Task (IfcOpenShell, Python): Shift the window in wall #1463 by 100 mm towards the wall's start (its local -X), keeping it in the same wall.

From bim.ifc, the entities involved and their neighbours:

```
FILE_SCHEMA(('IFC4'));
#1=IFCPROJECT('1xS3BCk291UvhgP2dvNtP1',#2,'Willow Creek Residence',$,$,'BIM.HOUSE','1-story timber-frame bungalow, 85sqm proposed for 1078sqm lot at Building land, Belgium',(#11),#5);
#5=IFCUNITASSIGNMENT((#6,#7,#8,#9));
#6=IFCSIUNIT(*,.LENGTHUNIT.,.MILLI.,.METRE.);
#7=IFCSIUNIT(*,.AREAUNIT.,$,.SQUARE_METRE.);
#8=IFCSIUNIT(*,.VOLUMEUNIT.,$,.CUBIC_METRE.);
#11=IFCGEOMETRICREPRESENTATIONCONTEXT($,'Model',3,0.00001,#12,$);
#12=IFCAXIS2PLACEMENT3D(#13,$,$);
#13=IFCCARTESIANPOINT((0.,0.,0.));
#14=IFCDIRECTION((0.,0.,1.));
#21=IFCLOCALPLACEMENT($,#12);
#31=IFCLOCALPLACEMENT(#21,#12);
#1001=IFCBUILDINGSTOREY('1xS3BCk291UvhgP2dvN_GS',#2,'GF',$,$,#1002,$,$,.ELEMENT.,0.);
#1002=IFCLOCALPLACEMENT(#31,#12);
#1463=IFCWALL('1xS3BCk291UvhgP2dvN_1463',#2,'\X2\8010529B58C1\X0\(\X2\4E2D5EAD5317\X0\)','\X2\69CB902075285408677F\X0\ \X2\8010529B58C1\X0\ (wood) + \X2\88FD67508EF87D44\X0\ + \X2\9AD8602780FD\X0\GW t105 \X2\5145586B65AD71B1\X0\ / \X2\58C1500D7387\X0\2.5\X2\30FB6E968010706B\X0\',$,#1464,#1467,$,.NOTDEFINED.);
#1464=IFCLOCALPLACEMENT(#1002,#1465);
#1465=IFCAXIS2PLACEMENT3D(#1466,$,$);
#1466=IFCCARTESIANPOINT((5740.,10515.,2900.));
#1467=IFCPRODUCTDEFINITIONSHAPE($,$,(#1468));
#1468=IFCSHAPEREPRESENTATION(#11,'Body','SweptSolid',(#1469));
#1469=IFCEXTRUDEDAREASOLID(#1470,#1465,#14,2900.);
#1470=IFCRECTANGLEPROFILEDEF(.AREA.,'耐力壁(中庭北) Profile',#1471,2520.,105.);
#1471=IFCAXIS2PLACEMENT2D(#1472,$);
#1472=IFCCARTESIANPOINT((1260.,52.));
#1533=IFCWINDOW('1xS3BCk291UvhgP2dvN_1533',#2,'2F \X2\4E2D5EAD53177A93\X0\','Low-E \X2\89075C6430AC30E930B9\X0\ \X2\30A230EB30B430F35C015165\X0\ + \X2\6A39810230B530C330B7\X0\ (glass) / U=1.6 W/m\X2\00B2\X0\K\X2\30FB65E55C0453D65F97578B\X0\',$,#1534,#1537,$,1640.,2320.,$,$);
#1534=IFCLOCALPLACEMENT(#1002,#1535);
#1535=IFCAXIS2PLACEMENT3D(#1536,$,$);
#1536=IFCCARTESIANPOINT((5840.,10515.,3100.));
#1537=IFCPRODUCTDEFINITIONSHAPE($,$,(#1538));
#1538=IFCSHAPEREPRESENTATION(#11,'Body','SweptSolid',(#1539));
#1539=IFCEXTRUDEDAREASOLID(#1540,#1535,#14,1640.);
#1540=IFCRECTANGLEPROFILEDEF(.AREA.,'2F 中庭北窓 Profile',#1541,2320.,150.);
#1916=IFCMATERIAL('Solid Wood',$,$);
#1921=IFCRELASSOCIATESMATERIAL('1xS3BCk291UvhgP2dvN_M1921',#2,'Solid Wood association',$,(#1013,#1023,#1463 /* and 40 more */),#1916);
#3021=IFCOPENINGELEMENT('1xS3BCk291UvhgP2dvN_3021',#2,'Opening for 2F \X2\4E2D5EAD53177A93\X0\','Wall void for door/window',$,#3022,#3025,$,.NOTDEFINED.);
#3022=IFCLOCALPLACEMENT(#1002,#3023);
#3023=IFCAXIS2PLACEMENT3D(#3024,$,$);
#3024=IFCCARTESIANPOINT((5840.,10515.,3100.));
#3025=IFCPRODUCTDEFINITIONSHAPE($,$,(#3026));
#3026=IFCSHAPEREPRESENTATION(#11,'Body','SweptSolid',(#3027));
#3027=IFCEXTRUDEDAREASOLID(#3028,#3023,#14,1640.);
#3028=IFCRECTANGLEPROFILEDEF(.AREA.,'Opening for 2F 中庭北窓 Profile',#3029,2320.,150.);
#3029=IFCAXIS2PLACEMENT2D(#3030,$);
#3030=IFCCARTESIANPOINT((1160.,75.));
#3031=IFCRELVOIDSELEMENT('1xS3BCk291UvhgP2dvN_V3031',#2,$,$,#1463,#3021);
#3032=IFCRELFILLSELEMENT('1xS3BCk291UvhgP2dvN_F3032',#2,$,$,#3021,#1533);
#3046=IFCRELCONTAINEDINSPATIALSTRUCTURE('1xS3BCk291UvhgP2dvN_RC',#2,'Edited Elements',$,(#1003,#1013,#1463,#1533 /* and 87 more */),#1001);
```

```python
import ifcopenshell
import ifcopenshell.api.geometry
import ifcopenshell.util.placement
import ifcopenshell.util.unit

model = ifcopenshell.open("bim.ifc")
unit_scale = ifcopenshell.util.unit.calculate_unit_scale(model)

window = model.by_guid("1xS3BCk291UvhgP2dvN_1533")
opening = window.FillsVoids[0].RelatingOpeningElement
wall = opening.VoidsElements[0].RelatingBuildingElement

wall_matrix = ifcopenshell.util.placement.get_local_placement(wall.ObjectPlacement)
shift = wall_matrix[:3, 0] * -0.1 / unit_scale
before = ifcopenshell.util.placement.get_local_placement(window.ObjectPlacement)[:3, 3].copy()

# The window is not placed relative to its opening, so move both.
for product in (opening, window):
    matrix = ifcopenshell.util.placement.get_local_placement(product.ObjectPlacement)
    matrix[:3, 3] += shift
    ifcopenshell.api.geometry.edit_object_placement(model, product=product, matrix=matrix, is_si=False)

after = ifcopenshell.util.placement.get_local_placement(window.ObjectPlacement)[:3, 3]
print("window moved by", (after - before).round(3) + 0.0)

model.write("bim_rev.ifc")
```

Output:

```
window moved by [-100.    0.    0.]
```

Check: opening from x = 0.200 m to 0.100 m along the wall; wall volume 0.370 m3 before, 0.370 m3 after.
